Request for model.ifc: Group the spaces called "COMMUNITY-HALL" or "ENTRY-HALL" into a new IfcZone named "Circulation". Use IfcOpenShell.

First a look at what the model holds.

```python
import ifcopenshell

model = ifcopenshell.open("model.ifc")
print(model.schema)
seen = {}
for space in model.by_type("IfcSpace"):
    seen[space.Name] = seen.get(space.Name, 0) + 1
for name, count in sorted(seen.items(), key=str):
    print(count, "x", name)
print("zones:", [z.Name for z in model.by_type("IfcZone")][:20])
```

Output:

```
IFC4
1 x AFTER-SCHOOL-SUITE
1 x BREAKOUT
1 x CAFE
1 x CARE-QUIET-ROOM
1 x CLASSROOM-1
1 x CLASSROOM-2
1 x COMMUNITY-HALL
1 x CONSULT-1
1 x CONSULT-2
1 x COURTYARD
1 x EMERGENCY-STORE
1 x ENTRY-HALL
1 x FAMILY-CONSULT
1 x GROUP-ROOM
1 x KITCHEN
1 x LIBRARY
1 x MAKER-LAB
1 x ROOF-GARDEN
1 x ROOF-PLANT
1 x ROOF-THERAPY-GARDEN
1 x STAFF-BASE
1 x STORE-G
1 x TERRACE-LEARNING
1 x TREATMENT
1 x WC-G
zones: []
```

```python
import ifcopenshell
import ifcopenshell.api.group
import ifcopenshell.api.root

model = ifcopenshell.open("model.ifc")

names = {"COMMUNITY-HALL", "ENTRY-HALL"}
spaces = [s for s in model.by_type("IfcSpace") if s.Name in names]

zone = ifcopenshell.api.root.create_entity(model, ifc_class="IfcZone", name="Circulation")
ifcopenshell.api.group.assign_group(model, products=spaces, group=zone)
print(len(spaces), "spaces in", zone.Name)

model.write("model_updated.ifc")
```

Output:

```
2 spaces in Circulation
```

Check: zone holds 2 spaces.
